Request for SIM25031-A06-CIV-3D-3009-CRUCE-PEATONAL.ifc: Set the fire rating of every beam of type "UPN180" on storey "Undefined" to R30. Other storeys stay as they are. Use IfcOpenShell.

First a look at what the model holds.

```python
import ifcopenshell
import ifcopenshell.util.element

model = ifcopenshell.open("SIM25031-A06-CIV-3D-3009-CRUCE-PEATONAL.ifc")
print(model.schema)
storey = next(s for s in model.by_type("IfcBuildingStorey") if s.Name == "Undefined")
beams = [e for e in ifcopenshell.util.element.get_decomposition(storey) if e.is_a("IfcBeam")]
seen = {}
for e in beams:
    element_type = ifcopenshell.util.element.get_type(e)
    key = (element_type.Name if element_type != e and element_type else None, ifcopenshell.util.element.get_pset(e, "Pset_BeamCommon", "FireRating"))
    seen[key] = seen.get(key, 0) + 1
for (name, value), count in sorted(seen.items(), key=str):
    print(count, "x", name, "|", value)
```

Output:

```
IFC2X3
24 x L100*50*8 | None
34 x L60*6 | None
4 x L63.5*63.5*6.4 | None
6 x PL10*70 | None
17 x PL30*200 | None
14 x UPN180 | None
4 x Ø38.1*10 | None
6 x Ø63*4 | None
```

```python
import ifcopenshell
import ifcopenshell.api.pset
import ifcopenshell.util.element

model = ifcopenshell.open("SIM25031-A06-CIV-3D-3009-CRUCE-PEATONAL.ifc")

storey = next(s for s in model.by_type("IfcBuildingStorey") if s.Name == "Undefined")
beams = [e for e in ifcopenshell.util.element.get_decomposition(storey) if e.is_a("IfcBeam")]

count = 0
for e in beams:
    element_type = ifcopenshell.util.element.get_type(e)
    if element_type in (None, e) or element_type.Name != "UPN180":
        continue
    found = ifcopenshell.util.element.get_pset(e, "Pset_BeamCommon", should_inherit=False)
    if found:
        pset = model.by_id(found["id"])
        if len(ifcopenshell.util.element.get_elements_by_pset(pset)) > 1:
            pset = ifcopenshell.api.pset.unshare_pset(model, products=[e], pset=pset)[0]
    else:
        pset = ifcopenshell.api.pset.add_pset(model, product=e, name="Pset_BeamCommon")
    ifcopenshell.api.pset.edit_pset(model, pset=pset, properties={"FireRating": "R30"})
    count += 1

print(count, "beams updated")

model.write("SIM25031-A06-CIV-3D-3009-CRUCE-PEATONAL_rev.ifc")
```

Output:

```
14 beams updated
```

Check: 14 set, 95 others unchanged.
